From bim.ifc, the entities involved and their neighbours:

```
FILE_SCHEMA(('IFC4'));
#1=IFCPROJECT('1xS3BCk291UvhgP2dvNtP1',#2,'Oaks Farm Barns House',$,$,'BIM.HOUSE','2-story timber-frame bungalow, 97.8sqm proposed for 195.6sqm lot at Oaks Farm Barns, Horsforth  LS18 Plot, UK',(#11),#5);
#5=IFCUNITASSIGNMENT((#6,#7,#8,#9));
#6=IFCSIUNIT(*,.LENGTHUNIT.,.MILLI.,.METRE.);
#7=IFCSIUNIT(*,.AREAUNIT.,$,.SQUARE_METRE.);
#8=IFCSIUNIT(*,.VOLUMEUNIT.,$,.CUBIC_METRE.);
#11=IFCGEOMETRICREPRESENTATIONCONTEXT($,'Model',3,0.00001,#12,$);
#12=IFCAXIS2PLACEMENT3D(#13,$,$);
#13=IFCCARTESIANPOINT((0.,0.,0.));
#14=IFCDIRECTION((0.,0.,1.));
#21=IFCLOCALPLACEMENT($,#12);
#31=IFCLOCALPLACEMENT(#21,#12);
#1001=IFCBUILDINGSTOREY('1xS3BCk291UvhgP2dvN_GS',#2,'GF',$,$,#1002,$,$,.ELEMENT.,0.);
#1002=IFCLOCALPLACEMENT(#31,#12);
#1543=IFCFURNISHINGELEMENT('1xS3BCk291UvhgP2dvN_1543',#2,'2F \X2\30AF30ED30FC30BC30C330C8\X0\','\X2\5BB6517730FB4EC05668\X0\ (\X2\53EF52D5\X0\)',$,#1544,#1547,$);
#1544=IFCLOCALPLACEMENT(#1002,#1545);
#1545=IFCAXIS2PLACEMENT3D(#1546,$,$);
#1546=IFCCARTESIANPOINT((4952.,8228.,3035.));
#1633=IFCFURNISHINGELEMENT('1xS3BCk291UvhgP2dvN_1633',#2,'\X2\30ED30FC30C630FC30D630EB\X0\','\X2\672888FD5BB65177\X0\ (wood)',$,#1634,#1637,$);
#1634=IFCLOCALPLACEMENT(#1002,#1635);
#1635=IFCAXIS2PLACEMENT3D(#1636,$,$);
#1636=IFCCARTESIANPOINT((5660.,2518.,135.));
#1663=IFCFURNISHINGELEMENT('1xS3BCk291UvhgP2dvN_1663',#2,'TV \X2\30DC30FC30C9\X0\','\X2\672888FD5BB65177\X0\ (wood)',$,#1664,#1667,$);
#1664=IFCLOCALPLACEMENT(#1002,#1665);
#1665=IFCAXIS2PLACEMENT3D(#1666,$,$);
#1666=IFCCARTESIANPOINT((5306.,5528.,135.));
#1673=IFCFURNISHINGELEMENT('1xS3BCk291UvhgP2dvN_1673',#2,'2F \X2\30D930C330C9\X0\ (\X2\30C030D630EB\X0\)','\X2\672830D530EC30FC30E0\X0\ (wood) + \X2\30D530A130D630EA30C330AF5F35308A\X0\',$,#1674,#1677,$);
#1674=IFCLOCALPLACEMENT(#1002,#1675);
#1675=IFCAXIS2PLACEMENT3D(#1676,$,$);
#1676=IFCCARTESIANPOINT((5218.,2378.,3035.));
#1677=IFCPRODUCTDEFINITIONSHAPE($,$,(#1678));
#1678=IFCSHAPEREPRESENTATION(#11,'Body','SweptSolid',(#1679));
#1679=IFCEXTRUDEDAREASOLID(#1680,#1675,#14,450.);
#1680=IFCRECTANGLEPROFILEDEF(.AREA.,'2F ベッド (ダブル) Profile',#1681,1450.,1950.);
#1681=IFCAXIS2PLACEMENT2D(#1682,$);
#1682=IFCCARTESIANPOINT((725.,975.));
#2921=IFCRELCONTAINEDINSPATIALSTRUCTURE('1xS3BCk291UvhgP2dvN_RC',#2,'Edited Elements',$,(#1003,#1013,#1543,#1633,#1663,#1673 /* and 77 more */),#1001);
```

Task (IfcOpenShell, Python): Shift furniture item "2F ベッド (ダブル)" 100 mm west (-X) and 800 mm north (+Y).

```python
import ifcopenshell
import ifcopenshell.api.geometry
import ifcopenshell.util.placement

model = ifcopenshell.open("bim.ifc")

item = model.by_guid("1xS3BCk291UvhgP2dvN_1673")
matrix = ifcopenshell.util.placement.get_local_placement(item.ObjectPlacement)
matrix[0, 3] -= 100.0
matrix[1, 3] += 800.0
ifcopenshell.api.geometry.edit_object_placement(model, product=item, matrix=matrix, is_si=False)

print(ifcopenshell.util.placement.get_local_placement(item.ObjectPlacement).round(3) + 0.0)

model.write("bim_v2.ifc")
```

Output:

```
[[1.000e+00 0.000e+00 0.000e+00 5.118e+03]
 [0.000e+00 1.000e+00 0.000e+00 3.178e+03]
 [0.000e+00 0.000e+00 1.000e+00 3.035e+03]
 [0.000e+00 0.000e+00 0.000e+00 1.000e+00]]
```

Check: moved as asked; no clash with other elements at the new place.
